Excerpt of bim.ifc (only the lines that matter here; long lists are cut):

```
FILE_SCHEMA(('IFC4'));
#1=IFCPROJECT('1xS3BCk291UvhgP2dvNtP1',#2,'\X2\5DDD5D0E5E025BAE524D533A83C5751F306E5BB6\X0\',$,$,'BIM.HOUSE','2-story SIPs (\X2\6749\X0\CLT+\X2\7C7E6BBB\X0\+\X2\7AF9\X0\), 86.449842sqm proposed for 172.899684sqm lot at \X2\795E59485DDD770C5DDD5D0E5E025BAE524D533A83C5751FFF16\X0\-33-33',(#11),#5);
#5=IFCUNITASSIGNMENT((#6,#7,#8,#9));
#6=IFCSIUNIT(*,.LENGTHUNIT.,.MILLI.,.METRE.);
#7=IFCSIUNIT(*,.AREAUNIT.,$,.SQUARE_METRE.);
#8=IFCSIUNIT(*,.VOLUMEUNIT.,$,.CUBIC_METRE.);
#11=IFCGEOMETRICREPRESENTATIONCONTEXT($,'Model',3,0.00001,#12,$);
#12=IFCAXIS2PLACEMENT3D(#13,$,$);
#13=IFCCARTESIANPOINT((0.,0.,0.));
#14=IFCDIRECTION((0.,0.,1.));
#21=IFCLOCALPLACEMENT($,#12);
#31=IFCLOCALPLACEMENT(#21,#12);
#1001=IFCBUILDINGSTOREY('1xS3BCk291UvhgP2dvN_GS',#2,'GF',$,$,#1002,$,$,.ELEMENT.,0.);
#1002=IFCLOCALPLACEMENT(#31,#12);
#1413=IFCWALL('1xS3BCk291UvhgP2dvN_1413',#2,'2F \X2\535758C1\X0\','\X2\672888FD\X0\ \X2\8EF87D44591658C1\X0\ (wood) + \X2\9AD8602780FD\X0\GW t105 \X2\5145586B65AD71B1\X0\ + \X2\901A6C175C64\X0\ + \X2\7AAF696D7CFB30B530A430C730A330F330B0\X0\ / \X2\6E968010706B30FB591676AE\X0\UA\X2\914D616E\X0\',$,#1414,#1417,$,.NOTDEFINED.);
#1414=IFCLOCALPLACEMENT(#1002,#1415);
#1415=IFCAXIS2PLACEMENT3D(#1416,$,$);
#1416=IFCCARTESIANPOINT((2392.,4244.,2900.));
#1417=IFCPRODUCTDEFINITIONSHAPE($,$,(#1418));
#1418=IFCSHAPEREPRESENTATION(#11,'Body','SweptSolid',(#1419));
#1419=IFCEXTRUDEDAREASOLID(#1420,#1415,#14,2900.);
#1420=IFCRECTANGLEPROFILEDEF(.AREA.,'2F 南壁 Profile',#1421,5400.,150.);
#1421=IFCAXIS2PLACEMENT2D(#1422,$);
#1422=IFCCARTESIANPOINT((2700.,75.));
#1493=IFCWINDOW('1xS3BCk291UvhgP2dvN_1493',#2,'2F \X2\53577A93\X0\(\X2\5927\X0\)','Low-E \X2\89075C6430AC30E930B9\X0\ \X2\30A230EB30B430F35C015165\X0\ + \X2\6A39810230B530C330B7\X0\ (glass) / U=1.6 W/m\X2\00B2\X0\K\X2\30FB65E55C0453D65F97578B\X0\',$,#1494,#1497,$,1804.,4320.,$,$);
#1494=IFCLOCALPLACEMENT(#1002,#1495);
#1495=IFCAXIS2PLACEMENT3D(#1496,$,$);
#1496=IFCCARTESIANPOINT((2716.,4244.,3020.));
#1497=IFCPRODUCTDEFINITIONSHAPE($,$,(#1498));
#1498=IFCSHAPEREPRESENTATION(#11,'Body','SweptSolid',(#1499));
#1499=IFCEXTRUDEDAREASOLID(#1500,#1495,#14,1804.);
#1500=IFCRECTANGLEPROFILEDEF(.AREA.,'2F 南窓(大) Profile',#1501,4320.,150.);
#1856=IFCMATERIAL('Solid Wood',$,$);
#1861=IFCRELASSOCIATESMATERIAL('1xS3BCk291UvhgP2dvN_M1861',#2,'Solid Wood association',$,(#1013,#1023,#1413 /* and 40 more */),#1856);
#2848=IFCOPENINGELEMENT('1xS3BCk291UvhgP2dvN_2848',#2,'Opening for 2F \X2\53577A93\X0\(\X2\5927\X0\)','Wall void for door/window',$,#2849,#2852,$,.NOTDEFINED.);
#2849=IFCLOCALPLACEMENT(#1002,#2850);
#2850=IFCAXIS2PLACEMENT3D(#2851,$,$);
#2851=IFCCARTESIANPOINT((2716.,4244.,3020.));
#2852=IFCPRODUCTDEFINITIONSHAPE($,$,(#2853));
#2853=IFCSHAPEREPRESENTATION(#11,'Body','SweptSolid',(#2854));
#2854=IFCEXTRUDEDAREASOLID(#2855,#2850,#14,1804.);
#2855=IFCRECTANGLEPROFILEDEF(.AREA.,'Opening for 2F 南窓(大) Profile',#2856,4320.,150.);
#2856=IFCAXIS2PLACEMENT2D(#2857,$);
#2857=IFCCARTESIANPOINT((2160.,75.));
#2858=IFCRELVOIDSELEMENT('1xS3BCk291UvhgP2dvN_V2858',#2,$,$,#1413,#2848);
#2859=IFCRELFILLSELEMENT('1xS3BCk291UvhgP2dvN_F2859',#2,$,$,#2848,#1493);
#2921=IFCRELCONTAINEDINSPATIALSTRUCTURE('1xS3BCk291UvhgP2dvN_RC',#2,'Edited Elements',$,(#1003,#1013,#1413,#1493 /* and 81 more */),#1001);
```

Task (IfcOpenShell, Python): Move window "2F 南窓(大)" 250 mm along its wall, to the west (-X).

```python
import ifcopenshell
import ifcopenshell.api.geometry
import ifcopenshell.util.placement

model = ifcopenshell.open("bim.ifc")

window = model.by_guid("1xS3BCk291UvhgP2dvN_1493")
opening = window.FillsVoids[0].RelatingOpeningElement
wall = opening.VoidsElements[0].RelatingBuildingElement

wall_matrix = ifcopenshell.util.placement.get_local_placement(wall.ObjectPlacement)
shift = wall_matrix[:3, 0] * -250.0
before = ifcopenshell.util.placement.get_local_placement(window.ObjectPlacement)[:3, 3].copy()

# The window is not placed relative to its opening, so move both.
for product in (opening, window):
    matrix = ifcopenshell.util.placement.get_local_placement(product.ObjectPlacement)
    matrix[:3, 3] += shift
    ifcopenshell.api.geometry.edit_object_placement(model, product=product, matrix=matrix, is_si=False)

after = ifcopenshell.util.placement.get_local_placement(window.ObjectPlacement)[:3, 3]
print("window moved by", (after - before).round(3) + 0.0)

model.write("bim_v2.ifc")
```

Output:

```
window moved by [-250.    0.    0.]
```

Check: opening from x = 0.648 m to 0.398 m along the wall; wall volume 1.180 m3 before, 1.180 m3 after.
